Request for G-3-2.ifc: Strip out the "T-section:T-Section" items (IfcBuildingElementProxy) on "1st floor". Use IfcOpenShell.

First a look at what the model holds.

```python
import ifcopenshell
import ifcopenshell.util.element

model = ifcopenshell.open("G-3-2.ifc")
print(model.schema)
storey = next(s for s in model.by_type("IfcBuildingStorey") if s.Name == "1st floor")
proxies = [e for e in ifcopenshell.util.element.get_decomposition(storey) if e.is_a("IfcBuildingElementProxy")]
seen = {}
for e in proxies:
    element_type = ifcopenshell.util.element.get_type(e)
    name = element_type.Name if element_type not in (None, e) else None
    seen[name] = seen.get(name, 0) + 1
for name, count in sorted(seen.items(), key=str):
    print(count, "x", name)
```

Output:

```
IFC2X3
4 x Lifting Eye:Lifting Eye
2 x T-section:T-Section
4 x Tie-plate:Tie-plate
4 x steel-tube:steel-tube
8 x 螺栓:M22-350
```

```python
import ifcopenshell
import ifcopenshell.api.root
import ifcopenshell.util.element

model = ifcopenshell.open("G-3-2.ifc")

storey = next(s for s in model.by_type("IfcBuildingStorey") if s.Name == "1st floor")
proxies = [e for e in ifcopenshell.util.element.get_decomposition(storey) if e.is_a("IfcBuildingElementProxy")]
targets = [e for e in proxies if (t := ifcopenshell.util.element.get_type(e)) not in (None, e) and t.Name == "T-section:T-Section"]

for e in targets:
    ifcopenshell.api.root.remove_product(model, product=e)
print(len(targets), "removed")

model.write("G-3-2_v2.ifc")
```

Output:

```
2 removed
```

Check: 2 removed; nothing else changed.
